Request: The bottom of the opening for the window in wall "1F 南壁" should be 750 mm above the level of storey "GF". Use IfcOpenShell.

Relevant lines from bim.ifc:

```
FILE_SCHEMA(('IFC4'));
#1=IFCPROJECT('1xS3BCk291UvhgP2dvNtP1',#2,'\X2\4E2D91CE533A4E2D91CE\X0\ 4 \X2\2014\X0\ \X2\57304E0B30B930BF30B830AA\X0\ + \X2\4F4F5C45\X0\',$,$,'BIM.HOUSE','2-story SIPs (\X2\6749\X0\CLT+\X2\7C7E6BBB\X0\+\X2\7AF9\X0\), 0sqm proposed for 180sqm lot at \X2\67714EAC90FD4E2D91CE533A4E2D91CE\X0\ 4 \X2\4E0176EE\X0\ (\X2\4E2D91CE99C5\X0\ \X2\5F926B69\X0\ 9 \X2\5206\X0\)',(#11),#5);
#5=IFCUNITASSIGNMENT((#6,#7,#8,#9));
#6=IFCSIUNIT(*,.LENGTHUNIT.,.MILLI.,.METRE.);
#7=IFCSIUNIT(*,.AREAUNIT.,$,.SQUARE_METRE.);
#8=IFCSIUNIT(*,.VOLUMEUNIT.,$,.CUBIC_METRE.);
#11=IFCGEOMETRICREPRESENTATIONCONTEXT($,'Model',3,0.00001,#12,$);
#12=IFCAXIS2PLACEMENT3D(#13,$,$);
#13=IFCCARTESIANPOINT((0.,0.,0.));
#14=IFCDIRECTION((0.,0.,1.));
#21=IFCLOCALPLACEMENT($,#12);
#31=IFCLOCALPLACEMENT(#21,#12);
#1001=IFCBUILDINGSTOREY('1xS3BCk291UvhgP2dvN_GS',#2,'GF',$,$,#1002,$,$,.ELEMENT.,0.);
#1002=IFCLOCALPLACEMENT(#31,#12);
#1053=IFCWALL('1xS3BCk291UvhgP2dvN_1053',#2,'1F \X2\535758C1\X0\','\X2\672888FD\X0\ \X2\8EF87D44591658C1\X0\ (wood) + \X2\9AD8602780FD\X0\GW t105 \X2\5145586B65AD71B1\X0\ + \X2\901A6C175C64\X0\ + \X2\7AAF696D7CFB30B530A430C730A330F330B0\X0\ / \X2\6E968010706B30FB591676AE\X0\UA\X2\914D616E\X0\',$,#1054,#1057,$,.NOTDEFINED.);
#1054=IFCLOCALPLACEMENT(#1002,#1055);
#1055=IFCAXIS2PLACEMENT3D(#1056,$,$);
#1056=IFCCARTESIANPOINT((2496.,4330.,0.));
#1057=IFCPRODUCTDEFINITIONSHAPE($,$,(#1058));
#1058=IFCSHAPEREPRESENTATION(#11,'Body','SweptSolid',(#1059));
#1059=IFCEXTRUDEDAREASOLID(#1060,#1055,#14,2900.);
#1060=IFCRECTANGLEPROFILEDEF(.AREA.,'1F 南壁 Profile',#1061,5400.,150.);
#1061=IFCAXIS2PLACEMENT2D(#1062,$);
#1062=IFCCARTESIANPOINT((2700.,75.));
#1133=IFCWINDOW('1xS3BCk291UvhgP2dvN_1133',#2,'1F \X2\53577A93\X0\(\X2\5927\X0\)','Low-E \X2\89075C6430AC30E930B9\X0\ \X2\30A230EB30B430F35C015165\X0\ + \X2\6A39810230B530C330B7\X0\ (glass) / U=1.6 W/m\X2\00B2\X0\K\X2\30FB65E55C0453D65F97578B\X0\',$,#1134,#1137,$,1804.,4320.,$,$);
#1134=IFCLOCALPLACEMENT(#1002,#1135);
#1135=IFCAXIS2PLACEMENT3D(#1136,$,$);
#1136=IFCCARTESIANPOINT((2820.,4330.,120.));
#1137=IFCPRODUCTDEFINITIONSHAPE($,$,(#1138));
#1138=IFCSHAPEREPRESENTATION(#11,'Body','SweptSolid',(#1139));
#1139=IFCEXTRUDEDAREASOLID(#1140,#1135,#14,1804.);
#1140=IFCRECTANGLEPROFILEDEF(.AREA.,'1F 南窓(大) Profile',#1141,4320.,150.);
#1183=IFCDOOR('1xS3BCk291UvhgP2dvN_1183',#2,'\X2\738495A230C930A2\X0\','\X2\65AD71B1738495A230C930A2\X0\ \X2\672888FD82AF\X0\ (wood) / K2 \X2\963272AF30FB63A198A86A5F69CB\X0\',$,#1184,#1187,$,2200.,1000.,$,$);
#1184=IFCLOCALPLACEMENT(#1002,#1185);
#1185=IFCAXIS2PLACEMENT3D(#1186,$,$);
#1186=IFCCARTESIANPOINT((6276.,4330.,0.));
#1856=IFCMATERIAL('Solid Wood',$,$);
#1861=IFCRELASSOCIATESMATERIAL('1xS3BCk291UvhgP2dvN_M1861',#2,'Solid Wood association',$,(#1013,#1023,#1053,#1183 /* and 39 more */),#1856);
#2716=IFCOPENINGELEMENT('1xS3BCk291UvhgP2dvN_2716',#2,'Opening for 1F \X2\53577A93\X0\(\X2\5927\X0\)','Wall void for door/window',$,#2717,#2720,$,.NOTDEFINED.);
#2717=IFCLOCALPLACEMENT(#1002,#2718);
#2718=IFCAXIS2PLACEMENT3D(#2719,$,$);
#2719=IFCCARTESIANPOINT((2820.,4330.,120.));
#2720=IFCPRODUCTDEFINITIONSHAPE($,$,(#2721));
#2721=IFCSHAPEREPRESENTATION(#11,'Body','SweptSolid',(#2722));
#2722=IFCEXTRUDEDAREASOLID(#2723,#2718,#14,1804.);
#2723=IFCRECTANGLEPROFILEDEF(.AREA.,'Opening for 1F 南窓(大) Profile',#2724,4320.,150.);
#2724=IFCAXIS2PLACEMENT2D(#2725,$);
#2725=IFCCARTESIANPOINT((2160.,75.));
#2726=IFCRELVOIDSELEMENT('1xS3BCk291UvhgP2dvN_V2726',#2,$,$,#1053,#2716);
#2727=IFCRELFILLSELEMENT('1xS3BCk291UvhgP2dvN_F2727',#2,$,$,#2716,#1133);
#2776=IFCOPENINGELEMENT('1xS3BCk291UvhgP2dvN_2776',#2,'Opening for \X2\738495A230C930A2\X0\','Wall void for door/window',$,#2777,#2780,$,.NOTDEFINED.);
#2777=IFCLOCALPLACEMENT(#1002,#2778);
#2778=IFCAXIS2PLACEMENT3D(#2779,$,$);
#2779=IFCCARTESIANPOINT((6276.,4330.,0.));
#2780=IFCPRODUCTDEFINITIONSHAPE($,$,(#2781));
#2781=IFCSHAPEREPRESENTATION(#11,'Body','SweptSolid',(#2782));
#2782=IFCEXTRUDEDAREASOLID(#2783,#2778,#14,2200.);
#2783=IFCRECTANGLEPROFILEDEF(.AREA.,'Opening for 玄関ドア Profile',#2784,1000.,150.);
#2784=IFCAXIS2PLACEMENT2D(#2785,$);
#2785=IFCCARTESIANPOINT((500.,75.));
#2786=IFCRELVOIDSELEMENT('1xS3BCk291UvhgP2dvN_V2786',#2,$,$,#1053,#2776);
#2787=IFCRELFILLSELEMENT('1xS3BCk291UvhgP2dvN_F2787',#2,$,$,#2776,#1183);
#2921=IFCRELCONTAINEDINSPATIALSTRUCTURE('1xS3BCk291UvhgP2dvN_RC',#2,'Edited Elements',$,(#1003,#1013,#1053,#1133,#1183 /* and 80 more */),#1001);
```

```python
import numpy as np
import ifcopenshell
import ifcopenshell.api.geometry
import ifcopenshell.geom
import ifcopenshell.util.element
import ifcopenshell.util.placement
import ifcopenshell.util.shape
import ifcopenshell.util.unit

model = ifcopenshell.open("bim.ifc")
unit_scale = ifcopenshell.util.unit.calculate_unit_scale(model)

window = model.by_id(1133)
opening = window.FillsVoids[0].RelatingOpeningElement
storey = ifcopenshell.util.element.get_container(window, ifc_class="IfcBuildingStorey")
level = ifcopenshell.util.placement.get_local_placement(storey.ObjectPlacement)[2, 3]

# The opening's origin need not be at the sill, so measure its lowest point.
shape = ifcopenshell.geom.create_shape(ifcopenshell.geom.settings(), opening)
bottom = ifcopenshell.util.shape.get_shape_bottom_elevation(shape, shape.geometry) / unit_scale
dz = level + 0.75 / unit_scale - bottom

shift = np.array([0.0, 0.0, dz])
# The window is not placed relative to its opening, so move both.
for product in (opening, window):
    matrix = ifcopenshell.util.placement.get_local_placement(product.ObjectPlacement)
    matrix[:3, 3] += shift
    ifcopenshell.api.geometry.edit_object_placement(model, product=product, matrix=matrix, is_si=False)

print(f"moved by {dz * unit_scale:+.3f} m")

model.write("bim_edited.ifc")
```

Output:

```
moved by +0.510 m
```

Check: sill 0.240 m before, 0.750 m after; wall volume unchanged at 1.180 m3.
